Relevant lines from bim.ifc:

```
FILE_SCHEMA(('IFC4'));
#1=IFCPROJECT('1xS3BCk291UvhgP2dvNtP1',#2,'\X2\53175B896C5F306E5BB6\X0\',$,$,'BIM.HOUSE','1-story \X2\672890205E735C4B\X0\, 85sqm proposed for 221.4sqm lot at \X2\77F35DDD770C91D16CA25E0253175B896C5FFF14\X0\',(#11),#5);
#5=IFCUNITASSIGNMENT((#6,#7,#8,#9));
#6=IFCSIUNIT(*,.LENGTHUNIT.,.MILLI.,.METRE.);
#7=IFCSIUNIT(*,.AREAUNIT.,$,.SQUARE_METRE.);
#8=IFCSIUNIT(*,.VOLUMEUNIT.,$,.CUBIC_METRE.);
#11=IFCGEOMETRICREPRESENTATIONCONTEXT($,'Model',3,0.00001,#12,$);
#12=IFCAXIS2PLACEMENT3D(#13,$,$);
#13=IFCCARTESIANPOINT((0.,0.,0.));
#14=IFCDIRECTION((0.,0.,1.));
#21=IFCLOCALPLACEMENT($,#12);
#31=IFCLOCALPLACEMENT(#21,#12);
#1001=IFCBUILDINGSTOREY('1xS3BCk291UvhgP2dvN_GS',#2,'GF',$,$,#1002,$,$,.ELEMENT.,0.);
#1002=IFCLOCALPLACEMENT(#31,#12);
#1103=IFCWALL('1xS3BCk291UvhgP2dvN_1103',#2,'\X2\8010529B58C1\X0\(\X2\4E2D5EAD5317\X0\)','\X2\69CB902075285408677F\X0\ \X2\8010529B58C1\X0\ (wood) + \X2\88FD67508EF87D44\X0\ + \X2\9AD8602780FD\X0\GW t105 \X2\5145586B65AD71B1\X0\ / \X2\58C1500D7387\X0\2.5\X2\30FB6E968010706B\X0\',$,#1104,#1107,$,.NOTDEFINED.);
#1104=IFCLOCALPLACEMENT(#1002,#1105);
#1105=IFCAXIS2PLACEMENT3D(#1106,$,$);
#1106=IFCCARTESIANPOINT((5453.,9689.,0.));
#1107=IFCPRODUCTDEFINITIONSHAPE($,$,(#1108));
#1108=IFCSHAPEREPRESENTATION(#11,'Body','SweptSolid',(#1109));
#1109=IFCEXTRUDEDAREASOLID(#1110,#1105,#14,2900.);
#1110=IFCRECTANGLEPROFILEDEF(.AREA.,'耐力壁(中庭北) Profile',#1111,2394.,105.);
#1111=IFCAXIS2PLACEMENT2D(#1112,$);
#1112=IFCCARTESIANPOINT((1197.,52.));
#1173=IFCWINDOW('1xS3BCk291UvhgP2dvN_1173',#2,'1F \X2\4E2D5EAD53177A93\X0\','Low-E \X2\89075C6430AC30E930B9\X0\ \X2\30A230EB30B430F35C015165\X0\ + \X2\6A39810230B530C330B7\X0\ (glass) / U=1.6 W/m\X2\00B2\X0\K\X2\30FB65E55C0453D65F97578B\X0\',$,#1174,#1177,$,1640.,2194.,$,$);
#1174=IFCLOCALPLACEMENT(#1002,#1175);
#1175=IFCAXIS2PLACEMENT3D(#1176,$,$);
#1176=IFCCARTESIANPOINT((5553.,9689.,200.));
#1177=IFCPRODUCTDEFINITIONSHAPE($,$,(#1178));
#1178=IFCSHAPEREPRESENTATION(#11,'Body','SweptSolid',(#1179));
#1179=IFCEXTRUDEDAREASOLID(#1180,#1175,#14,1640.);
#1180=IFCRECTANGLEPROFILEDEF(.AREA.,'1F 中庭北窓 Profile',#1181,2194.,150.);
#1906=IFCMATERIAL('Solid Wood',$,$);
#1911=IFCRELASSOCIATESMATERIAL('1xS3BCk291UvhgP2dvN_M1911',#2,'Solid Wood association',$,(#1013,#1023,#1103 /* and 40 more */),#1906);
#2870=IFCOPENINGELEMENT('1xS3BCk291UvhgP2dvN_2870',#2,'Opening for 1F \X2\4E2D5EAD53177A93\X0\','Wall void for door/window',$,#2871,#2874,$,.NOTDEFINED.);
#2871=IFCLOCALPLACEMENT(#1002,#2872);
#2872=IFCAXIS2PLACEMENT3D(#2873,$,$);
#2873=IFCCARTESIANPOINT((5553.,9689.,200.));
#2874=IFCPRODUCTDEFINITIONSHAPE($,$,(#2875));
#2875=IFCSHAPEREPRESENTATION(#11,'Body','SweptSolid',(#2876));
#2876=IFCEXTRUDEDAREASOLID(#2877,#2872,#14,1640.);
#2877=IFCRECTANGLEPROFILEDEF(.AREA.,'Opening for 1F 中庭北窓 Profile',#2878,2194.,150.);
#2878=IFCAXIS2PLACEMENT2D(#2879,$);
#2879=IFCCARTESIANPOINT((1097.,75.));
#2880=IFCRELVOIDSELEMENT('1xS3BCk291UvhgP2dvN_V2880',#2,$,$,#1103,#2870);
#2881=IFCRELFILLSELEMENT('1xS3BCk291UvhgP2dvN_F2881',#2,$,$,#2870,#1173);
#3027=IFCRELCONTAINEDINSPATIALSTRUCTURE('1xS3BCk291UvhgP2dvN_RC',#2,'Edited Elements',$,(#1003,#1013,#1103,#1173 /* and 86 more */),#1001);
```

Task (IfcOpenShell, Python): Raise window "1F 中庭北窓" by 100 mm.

```python
import numpy as np
import ifcopenshell
import ifcopenshell.api.geometry
import ifcopenshell.util.placement
import ifcopenshell.util.unit

model = ifcopenshell.open("bim.ifc")
unit_scale = ifcopenshell.util.unit.calculate_unit_scale(model)

window = model.by_guid("1xS3BCk291UvhgP2dvN_1173")
opening = window.FillsVoids[0].RelatingOpeningElement
dz = 0.1 / unit_scale

shift = np.array([0.0, 0.0, dz])
# The window is not placed relative to its opening, so move both.
for product in (opening, window):
    matrix = ifcopenshell.util.placement.get_local_placement(product.ObjectPlacement)
    matrix[:3, 3] += shift
    ifcopenshell.api.geometry.edit_object_placement(model, product=product, matrix=matrix, is_si=False)

print(f"moved by {dz * unit_scale:+.3f} m")

model.write("bim_updated.ifc")
```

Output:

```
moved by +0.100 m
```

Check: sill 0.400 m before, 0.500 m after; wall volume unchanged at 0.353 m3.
